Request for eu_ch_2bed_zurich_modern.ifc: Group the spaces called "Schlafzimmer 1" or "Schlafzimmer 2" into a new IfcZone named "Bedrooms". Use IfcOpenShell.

First a look at what the model holds.

```python
import ifcopenshell

model = ifcopenshell.open("eu_ch_2bed_zurich_modern.ifc")
print(model.schema)
seen = {}
for space in model.by_type("IfcSpace"):
    seen[space.LongName] = seen.get(space.LongName, 0) + 1
for name, count in sorted(seen.items(), key=str):
    print(count, "x", name)
print("zones:", [z.Name for z in model.by_type("IfcZone")][:20])
```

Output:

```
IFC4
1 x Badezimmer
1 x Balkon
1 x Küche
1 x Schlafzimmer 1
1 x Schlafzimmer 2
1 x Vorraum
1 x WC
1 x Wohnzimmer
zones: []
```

```python
import ifcopenshell
import ifcopenshell.api.group
import ifcopenshell.api.root

model = ifcopenshell.open("eu_ch_2bed_zurich_modern.ifc")

names = {"Schlafzimmer 1", "Schlafzimmer 2"}
spaces = [s for s in model.by_type("IfcSpace") if s.LongName in names]

zone = ifcopenshell.api.root.create_entity(model, ifc_class="IfcZone", name="Bedrooms")
ifcopenshell.api.group.assign_group(model, products=spaces, group=zone)
print(len(spaces), "spaces in", zone.Name)

model.write("eu_ch_2bed_zurich_modern_v2.ifc")
```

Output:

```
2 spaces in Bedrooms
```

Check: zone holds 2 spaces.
